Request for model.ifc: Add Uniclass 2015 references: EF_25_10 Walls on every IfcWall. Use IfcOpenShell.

First a look at what the model holds.

```python
import ifcopenshell

model = ifcopenshell.open("model.ifc")
print(model.schema)
print("classifications:", [c.Name for c in model.by_type("IfcClassification")])
for ifc_class in ("IfcDoor", "IfcRoof", "IfcStair", "IfcWall", "IfcWindow"):
    print(ifc_class, len(model.by_type(ifc_class)))
```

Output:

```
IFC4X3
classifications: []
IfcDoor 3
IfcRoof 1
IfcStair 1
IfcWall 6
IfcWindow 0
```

```python
import ifcopenshell
import ifcopenshell.api.classification

model = ifcopenshell.open("model.ifc")

system = ifcopenshell.api.classification.add_classification(model, classification="Uniclass 2015")

codes = {
    "IfcWall": ("EF_25_10", "Walls"),
}
for ifc_class, (code, name) in codes.items():
    products = model.by_type(ifc_class)
    ifcopenshell.api.classification.add_reference(
        model, products=products, classification=system, identification=code, name=name
    )
    print(code, len(products))

model.write("model_rev.ifc")
```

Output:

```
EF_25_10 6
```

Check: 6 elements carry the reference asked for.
